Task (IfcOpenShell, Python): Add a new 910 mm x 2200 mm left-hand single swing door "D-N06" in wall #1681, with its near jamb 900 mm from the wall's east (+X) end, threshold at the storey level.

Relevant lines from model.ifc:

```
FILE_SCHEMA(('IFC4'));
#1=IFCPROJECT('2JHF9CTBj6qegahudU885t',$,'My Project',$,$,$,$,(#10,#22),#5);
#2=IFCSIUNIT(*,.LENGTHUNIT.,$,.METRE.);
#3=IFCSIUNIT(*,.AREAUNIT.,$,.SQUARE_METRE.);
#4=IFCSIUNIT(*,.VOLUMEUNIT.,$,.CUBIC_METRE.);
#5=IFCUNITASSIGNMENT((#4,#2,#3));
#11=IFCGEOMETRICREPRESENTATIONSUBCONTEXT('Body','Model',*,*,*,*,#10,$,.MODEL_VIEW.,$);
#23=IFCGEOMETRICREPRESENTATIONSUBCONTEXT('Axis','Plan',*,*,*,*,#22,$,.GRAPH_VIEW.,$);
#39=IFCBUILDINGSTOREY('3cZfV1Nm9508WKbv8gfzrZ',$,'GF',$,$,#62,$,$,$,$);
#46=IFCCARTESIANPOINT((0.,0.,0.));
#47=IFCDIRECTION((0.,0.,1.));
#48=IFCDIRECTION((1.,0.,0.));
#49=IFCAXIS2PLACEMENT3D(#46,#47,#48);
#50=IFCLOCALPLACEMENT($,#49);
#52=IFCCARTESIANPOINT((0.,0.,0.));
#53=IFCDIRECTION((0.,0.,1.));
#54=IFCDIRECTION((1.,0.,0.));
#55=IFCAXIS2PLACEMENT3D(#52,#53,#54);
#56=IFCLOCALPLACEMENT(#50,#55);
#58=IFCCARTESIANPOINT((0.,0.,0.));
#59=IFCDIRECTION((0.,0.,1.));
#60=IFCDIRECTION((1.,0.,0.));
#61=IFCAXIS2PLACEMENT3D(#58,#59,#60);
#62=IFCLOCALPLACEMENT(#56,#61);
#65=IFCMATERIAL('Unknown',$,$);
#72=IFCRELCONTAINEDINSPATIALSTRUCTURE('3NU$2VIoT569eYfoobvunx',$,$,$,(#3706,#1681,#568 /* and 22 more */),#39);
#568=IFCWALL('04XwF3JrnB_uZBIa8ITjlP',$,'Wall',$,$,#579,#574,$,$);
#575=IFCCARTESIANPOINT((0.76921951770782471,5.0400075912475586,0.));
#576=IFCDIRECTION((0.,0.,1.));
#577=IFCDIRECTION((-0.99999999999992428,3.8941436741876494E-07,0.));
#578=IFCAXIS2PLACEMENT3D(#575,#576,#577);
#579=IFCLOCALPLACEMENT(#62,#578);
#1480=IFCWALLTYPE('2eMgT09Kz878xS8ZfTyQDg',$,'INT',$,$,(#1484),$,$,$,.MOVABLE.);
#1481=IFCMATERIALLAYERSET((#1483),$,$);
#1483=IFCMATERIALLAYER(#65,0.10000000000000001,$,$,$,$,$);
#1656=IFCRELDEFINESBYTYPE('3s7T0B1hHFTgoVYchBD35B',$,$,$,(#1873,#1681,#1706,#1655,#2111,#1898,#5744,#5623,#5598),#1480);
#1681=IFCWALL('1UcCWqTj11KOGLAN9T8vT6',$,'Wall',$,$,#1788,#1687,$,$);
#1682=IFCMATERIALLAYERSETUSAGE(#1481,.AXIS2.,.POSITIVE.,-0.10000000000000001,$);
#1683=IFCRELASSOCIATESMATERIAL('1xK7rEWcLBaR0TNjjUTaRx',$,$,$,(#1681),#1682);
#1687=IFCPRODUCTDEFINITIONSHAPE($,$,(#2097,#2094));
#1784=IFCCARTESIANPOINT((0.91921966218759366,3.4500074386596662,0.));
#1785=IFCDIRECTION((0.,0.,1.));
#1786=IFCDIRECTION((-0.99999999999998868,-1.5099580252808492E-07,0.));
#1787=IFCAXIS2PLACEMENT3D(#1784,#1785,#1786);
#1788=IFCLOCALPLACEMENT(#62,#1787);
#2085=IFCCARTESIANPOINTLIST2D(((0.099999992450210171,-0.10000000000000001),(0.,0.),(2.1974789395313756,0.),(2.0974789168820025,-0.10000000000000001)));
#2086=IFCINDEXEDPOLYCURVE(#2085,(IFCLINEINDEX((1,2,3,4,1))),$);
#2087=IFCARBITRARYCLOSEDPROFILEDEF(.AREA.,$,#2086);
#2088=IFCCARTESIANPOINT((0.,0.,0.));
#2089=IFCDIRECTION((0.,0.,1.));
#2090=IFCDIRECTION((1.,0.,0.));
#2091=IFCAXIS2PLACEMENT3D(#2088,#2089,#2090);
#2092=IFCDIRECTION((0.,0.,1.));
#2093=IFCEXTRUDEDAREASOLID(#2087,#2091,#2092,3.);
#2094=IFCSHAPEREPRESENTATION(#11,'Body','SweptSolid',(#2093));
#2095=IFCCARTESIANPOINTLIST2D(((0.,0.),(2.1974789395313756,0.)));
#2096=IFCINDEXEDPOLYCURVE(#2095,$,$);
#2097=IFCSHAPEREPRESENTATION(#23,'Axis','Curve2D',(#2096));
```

```python
import numpy as np
import ifcopenshell
import ifcopenshell.api.feature
import ifcopenshell.api.geometry
import ifcopenshell.api.root
import ifcopenshell.api.spatial
import ifcopenshell.geom
import ifcopenshell.util.element
import ifcopenshell.util.placement
import ifcopenshell.util.representation
import ifcopenshell.util.shape
import ifcopenshell.util.unit

model = ifcopenshell.open("model.ifc")
unit_scale = ifcopenshell.util.unit.calculate_unit_scale(model)
settings = ifcopenshell.geom.settings()


def volume(element):
    """Net volume in cubic metres, openings subtracted."""
    shape = ifcopenshell.geom.create_shape(settings, element)
    return ifcopenshell.util.shape.get_volume(shape.geometry)


wall = model.by_guid("1UcCWqTj11KOGLAN9T8vT6")
storey = ifcopenshell.util.element.get_container(wall, ifc_class="IfcBuildingStorey")
context = ifcopenshell.util.representation.get_context(model, "Model", "Body", "MODEL_VIEW")
before = volume(wall)

width, height, from_end, sill = 0.91, 2.2, 0.9, 0.0  # metres

# The wall runs along its own X axis, and the end named is its -X end.
wall_shape = ifcopenshell.geom.create_shape(settings, wall)
x, y, z = ifcopenshell.util.shape.get_vertices(wall_shape.geometry).T
start = x.min() + from_end
face, thickness = float(y.min()), float(y.max() - y.min())
wall_matrix = ifcopenshell.util.placement.get_local_placement(wall.ObjectPlacement)
level = ifcopenshell.util.placement.get_local_placement(storey.ObjectPlacement)[2, 3]


def in_wall(x, y):
    """Placement at x, y metres in the wall's axes, at sill height."""
    matrix = wall_matrix.copy()
    matrix[:, 3] = wall_matrix @ np.array([x / unit_scale, y / unit_scale, 0.0, 1.0])
    matrix[2, 3] = level + sill / unit_scale
    return matrix


# Opening: a box that overshoots both wall faces by 50 mm.
opening = ifcopenshell.api.root.create_entity(model, ifc_class="IfcOpeningElement", predefined_type="OPENING")
box = ifcopenshell.api.geometry.add_wall_representation(
    model, context=context, length=width, height=height, thickness=thickness + 0.1
)
ifcopenshell.api.geometry.assign_representation(model, product=opening, representation=box)
ifcopenshell.api.geometry.edit_object_placement(model, product=opening, matrix=in_wall(start, face - 0.05), is_si=False)
ifcopenshell.api.feature.add_feature(model, feature=opening, element=wall)

door = ifcopenshell.api.root.create_entity(model, ifc_class="IfcDoor", name="D-N06", predefined_type="DOOR")
door.OverallWidth, door.OverallHeight = width / unit_scale, height / unit_scale
door.OperationType = "SINGLE_SWING_LEFT"
body = ifcopenshell.api.geometry.add_door_representation(
    model,
    context=context,
    overall_width=door.OverallWidth,
    overall_height=door.OverallHeight,
    operation_type="SINGLE_SWING_LEFT",
    lining_properties={"LiningDepth": thickness / unit_scale, "ThresholdDepth": thickness / unit_scale},
)
ifcopenshell.api.geometry.assign_representation(model, product=door, representation=body)
ifcopenshell.api.spatial.assign_container(model, products=[door], relating_structure=storey)
ifcopenshell.api.feature.add_filling(model, opening=opening, element=door)

# The lining spans the wall, so the door starts at the wall face.
ifcopenshell.api.geometry.edit_object_placement(model, product=door, matrix=in_wall(start, face), is_si=False)

after = volume(wall)

print(f"wall volume {before:.3f} -> {after:.3f} m3")

model.write("model_updated.ifc")
```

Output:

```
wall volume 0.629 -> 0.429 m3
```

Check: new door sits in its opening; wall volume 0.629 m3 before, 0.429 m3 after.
